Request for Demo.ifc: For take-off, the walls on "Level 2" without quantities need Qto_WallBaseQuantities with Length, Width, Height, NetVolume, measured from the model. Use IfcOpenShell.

First a look at what the model holds.

```python
import ifcopenshell
import ifcopenshell.util.element
import ifcopenshell.util.unit

model = ifcopenshell.open("Demo.ifc")
print(model.schema)
for unit_type in ("LENGTHUNIT", "AREAUNIT", "VOLUMEUNIT"):
    print(unit_type, ifcopenshell.util.unit.calculate_unit_scale(model, unit_type))
storey = next(s for s in model.by_type("IfcBuildingStorey") if s.Name == "Level 2")
walls = [e for e in ifcopenshell.util.element.get_decomposition(storey) if e.is_a("IfcWall")]
for e in sorted(walls, key=lambda e: e.id()):
    print(e.id(), e.is_a(), e.Name, list(ifcopenshell.util.element.get_psets(e, qtos_only=True)), sep=" | ")
```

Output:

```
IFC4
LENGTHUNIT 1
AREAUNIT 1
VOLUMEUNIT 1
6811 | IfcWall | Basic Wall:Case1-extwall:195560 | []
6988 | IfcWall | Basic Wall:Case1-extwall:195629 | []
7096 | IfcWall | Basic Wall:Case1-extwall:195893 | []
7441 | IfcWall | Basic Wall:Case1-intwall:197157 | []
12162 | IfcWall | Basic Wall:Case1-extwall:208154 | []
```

```python
import ifcopenshell
import ifcopenshell.api.pset
import ifcopenshell.geom
import ifcopenshell.util.element
import ifcopenshell.util.shape
import ifcopenshell.util.unit

model = ifcopenshell.open("Demo.ifc")
unit_scale = ifcopenshell.util.unit.calculate_unit_scale(model)
volume_scale = ifcopenshell.util.unit.calculate_unit_scale(model, "VOLUMEUNIT")
settings = ifcopenshell.geom.settings()

storey = next(s for s in model.by_type("IfcBuildingStorey") if s.Name == "Level 2")
walls = [e for e in ifcopenshell.util.element.get_decomposition(storey) if e.is_a("IfcWall")]

for e in sorted(walls, key=lambda e: e.id()):
    if ifcopenshell.util.element.get_psets(e, qtos_only=True, should_inherit=False):
        continue
    # Geometry comes back in metres, in the element's own axes.
    shape = ifcopenshell.geom.create_shape(settings, e)
    values = {
        "Length": ifcopenshell.util.shape.get_x(shape.geometry) / unit_scale,
        "Width": ifcopenshell.util.shape.get_y(shape.geometry) / unit_scale,
        "Height": ifcopenshell.util.shape.get_z(shape.geometry) / unit_scale,
        "NetVolume": ifcopenshell.util.shape.get_volume(shape.geometry) / volume_scale,
    }
    qto = ifcopenshell.api.pset.add_qto(model, product=e, name="Qto_WallBaseQuantities")
    ifcopenshell.api.pset.edit_qto(model, qto=qto, properties=values)
    print(e.id(), {k: round(v, 3) for k, v in values.items()})

model.write("Demo-out.ifc")
```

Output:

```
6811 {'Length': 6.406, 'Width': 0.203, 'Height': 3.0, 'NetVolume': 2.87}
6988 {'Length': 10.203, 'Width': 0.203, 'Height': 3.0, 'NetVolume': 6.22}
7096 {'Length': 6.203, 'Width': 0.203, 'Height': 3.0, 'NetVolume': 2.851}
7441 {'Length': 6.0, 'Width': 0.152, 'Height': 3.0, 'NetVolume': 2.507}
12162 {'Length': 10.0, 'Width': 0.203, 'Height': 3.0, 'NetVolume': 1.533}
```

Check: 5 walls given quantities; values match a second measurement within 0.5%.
